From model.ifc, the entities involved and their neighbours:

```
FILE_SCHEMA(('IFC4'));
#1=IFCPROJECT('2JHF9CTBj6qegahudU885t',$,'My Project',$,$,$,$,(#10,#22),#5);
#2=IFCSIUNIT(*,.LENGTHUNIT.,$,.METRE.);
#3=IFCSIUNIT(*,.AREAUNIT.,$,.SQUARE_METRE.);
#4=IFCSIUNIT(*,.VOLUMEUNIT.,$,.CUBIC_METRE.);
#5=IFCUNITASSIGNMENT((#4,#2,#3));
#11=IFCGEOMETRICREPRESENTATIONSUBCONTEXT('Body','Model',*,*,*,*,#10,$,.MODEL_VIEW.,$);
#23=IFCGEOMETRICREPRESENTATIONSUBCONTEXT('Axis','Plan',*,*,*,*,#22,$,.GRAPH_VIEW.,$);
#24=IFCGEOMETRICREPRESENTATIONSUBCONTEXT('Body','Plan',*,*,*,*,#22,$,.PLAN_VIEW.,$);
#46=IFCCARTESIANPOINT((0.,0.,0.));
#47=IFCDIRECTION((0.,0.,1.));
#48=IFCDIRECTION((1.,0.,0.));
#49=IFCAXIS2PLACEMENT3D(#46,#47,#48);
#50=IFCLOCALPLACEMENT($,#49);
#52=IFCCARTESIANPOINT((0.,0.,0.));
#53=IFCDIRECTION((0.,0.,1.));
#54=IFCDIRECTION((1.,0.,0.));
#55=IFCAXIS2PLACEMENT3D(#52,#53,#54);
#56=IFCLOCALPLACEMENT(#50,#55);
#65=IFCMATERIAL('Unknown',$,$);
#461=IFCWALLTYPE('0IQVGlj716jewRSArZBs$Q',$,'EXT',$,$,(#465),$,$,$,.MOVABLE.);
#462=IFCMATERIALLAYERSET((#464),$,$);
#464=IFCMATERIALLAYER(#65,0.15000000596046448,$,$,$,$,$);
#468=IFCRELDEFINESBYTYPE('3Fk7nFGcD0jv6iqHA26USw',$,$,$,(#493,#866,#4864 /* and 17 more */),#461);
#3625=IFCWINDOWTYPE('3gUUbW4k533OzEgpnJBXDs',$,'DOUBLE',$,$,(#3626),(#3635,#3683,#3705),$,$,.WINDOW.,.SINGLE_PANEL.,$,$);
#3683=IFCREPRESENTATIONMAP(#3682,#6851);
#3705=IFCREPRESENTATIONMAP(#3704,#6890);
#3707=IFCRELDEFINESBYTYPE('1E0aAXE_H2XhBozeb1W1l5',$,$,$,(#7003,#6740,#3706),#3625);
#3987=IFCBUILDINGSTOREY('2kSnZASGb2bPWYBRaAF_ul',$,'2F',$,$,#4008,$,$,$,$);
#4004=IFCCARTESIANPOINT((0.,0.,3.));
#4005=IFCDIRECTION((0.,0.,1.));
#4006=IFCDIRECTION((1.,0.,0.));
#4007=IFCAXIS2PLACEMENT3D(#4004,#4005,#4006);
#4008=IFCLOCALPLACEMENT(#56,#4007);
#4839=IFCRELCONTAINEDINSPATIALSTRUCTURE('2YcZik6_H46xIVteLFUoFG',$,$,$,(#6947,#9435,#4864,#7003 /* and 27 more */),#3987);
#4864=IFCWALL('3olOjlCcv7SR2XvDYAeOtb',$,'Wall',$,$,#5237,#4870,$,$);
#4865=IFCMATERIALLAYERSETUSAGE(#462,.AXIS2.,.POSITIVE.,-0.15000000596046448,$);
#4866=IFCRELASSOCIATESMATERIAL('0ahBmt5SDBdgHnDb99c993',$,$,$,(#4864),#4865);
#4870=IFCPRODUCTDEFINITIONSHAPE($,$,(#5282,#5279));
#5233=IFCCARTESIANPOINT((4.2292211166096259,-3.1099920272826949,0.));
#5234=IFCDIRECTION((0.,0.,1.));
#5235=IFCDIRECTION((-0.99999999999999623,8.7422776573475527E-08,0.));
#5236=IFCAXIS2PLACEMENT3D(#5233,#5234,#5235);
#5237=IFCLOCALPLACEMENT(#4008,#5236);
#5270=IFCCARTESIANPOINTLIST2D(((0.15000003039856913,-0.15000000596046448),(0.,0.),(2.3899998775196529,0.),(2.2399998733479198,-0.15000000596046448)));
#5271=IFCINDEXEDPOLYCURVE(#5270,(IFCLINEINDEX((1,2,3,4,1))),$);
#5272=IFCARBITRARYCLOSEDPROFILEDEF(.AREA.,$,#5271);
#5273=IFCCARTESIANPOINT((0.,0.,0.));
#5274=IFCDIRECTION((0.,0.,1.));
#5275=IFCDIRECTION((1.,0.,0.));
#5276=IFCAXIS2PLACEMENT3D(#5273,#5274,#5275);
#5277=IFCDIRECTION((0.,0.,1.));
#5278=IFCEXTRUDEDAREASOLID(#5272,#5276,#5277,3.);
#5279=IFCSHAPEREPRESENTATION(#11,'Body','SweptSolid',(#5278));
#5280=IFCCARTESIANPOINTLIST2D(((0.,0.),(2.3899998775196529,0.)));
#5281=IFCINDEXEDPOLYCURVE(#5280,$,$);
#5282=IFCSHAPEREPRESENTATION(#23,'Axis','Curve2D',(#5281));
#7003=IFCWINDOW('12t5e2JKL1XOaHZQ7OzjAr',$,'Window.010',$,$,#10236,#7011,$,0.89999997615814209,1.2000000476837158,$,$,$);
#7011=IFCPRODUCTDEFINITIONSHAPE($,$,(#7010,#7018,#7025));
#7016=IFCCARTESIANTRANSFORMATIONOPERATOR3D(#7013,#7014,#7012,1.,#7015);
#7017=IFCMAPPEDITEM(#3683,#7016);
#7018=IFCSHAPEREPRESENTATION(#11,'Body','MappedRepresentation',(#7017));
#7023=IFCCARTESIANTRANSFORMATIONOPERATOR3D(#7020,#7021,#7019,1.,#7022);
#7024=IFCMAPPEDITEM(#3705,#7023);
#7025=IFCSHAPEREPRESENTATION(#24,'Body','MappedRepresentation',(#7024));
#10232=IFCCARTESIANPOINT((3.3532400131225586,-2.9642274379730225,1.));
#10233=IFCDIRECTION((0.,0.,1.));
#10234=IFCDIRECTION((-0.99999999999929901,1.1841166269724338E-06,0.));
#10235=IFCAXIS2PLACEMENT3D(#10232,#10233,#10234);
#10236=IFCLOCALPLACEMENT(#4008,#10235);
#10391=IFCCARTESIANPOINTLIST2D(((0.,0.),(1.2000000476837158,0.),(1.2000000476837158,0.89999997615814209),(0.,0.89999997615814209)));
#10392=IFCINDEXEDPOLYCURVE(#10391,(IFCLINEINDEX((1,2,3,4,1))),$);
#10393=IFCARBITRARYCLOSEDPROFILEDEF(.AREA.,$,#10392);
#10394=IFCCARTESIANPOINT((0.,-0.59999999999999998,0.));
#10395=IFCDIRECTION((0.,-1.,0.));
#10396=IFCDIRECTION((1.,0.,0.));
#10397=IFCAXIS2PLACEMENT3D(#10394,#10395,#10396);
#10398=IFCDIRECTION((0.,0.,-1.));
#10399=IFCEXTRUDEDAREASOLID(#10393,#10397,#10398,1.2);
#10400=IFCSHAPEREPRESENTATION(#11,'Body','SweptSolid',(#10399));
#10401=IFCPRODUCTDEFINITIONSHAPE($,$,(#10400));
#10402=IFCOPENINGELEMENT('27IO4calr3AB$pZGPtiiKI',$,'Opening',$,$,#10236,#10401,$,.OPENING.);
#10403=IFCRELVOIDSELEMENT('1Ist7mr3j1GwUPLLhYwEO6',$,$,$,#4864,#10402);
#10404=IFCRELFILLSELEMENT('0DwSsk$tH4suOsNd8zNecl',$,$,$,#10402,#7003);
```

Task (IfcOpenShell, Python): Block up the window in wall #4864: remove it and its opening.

```python
import ifcopenshell
import ifcopenshell.api.feature
import ifcopenshell.api.root
import ifcopenshell.geom
import ifcopenshell.util.shape

model = ifcopenshell.open("model.ifc")
settings = ifcopenshell.geom.settings()


def volume(element):
    """Net volume in cubic metres, openings subtracted."""
    shape = ifcopenshell.geom.create_shape(settings, element)
    return ifcopenshell.util.shape.get_volume(shape.geometry)


window = model.by_guid("12t5e2JKL1XOaHZQ7OzjAr")
opening = window.FillsVoids[0].RelatingOpeningElement
wall = opening.VoidsElements[0].RelatingBuildingElement
before = volume(wall)

ifcopenshell.api.root.remove_product(model, product=window)
ifcopenshell.api.feature.remove_feature(model, feature=opening)

after = volume(wall)

print(f"wall volume {before:.3f} -> {after:.3f} m3")

model.write("model_rev.ifc")
```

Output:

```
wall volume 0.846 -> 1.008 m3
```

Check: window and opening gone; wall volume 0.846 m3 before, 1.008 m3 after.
